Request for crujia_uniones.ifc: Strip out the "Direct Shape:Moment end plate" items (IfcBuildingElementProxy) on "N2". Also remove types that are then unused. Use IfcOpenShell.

First a look at what the model holds.

```python
import ifcopenshell
import ifcopenshell.util.element

model = ifcopenshell.open("crujia_uniones.ifc")
print(model.schema)
storey = next(s for s in model.by_type("IfcBuildingStorey") if s.Name == "N2")
proxies = [e for e in ifcopenshell.util.element.get_decomposition(storey) if e.is_a("IfcBuildingElementProxy")]
seen = {}
for e in proxies:
    element_type = ifcopenshell.util.element.get_type(e)
    name = element_type.Name if element_type not in (None, e) else None
    seen[name] = seen.get(name, 0) + 1
for name, count in sorted(seen.items(), key=str):
    print(count, "x", name)
```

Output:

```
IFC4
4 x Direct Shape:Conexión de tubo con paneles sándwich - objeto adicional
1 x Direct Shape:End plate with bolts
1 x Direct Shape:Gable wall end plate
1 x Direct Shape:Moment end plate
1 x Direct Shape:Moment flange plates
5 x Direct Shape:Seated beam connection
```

```python
import ifcopenshell
import ifcopenshell.api.root
import ifcopenshell.util.element

model = ifcopenshell.open("crujia_uniones.ifc")

storey = next(s for s in model.by_type("IfcBuildingStorey") if s.Name == "N2")
proxies = [e for e in ifcopenshell.util.element.get_decomposition(storey) if e.is_a("IfcBuildingElementProxy")]
targets = [e for e in proxies if (t := ifcopenshell.util.element.get_type(e)) not in (None, e) and t.Name == "Direct Shape:Moment end plate"]
types = {ifcopenshell.util.element.get_type(e) for e in targets} - {None, *targets}

for e in targets:
    ifcopenshell.api.root.remove_product(model, product=e)
print(len(targets), "removed")

unused = [t for t in types if not ifcopenshell.util.element.get_types(t)]
for t in unused:
    ifcopenshell.api.root.remove_product(model, product=t)
print(len(unused), "unused types removed")

model.write("crujia_uniones_edited.ifc")
```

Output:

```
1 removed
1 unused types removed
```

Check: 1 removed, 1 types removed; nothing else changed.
